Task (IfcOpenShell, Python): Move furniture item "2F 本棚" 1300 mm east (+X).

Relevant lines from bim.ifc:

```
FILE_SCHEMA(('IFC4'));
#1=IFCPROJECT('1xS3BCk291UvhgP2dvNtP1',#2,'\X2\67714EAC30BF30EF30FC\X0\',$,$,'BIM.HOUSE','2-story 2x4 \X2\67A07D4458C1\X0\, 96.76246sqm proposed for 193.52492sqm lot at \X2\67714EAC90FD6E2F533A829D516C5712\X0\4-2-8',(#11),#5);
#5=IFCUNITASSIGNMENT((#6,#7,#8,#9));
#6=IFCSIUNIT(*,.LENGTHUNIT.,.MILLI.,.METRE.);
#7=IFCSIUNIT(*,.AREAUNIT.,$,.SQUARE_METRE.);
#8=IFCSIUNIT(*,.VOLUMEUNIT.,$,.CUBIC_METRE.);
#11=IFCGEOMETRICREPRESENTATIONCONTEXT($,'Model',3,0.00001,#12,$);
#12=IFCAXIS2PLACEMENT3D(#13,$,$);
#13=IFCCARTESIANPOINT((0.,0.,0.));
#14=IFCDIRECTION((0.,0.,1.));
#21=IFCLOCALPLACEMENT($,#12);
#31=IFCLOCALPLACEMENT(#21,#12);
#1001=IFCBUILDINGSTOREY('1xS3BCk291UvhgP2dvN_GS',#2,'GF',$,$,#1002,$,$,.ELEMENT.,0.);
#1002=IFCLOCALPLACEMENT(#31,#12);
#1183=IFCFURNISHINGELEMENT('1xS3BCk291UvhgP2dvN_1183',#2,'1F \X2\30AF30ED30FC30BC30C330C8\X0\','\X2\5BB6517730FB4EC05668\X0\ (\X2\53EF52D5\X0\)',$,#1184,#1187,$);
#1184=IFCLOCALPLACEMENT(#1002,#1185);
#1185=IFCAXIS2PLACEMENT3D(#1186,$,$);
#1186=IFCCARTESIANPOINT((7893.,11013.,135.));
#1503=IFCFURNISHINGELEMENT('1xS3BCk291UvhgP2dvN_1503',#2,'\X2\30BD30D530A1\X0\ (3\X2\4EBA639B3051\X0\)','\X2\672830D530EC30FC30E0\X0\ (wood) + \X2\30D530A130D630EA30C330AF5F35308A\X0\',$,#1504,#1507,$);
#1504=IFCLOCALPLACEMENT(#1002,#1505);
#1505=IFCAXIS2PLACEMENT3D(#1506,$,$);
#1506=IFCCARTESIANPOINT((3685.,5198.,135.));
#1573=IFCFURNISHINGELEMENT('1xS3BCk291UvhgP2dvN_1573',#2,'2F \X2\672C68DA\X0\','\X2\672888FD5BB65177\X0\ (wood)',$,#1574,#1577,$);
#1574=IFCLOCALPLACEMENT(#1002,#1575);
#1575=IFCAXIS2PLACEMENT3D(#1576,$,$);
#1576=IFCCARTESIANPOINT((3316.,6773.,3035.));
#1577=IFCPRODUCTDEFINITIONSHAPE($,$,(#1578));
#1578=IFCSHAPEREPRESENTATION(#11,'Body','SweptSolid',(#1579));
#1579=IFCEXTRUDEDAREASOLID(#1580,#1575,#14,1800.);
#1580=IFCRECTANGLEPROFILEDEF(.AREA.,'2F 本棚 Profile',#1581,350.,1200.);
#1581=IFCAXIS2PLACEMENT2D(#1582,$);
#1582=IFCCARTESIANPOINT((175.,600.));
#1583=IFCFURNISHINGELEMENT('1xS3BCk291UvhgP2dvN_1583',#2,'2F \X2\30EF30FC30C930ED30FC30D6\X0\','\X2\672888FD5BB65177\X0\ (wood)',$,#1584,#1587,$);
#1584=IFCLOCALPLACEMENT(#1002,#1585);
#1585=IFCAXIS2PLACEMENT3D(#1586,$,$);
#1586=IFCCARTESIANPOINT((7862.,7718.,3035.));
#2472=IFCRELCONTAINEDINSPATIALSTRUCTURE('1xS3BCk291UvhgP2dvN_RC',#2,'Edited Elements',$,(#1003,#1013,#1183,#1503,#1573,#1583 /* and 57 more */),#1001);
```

```python
import ifcopenshell
import ifcopenshell.api.geometry
import ifcopenshell.util.placement
import ifcopenshell.util.unit

model = ifcopenshell.open("bim.ifc")
unit_scale = ifcopenshell.util.unit.calculate_unit_scale(model)

item = model.by_guid("1xS3BCk291UvhgP2dvN_1573")
matrix = ifcopenshell.util.placement.get_local_placement(item.ObjectPlacement)
matrix[0, 3] += 1.3 / unit_scale
ifcopenshell.api.geometry.edit_object_placement(model, product=item, matrix=matrix, is_si=False)

print(ifcopenshell.util.placement.get_local_placement(item.ObjectPlacement).round(3) + 0.0)

model.write("bim_rev.ifc")
```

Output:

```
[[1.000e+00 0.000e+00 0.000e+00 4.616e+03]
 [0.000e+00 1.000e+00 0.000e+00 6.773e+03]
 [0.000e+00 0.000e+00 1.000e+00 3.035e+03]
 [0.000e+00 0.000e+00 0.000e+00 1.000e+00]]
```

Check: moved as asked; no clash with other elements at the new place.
